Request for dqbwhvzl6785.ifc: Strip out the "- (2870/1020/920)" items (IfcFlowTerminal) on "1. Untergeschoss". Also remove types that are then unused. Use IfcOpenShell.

First a look at what the model holds.

```python
import ifcopenshell
import ifcopenshell.util.element

model = ifcopenshell.open("dqbwhvzl6785.ifc")
print(model.schema)
storey = next(s for s in model.by_type("IfcBuildingStorey") if s.Name == "1. Untergeschoss")
terminals = [e for e in ifcopenshell.util.element.get_decomposition(storey) if e.is_a("IfcFlowTerminal")]
seen = {}
for e in terminals:
    element_type = ifcopenshell.util.element.get_type(e)
    name = element_type.Name if element_type not in (None, e) else None
    seen[name] = seen.get(name, 0) + 1
for name, count in sorted(seen.items(), key=str):
    print(count, "x", name)
```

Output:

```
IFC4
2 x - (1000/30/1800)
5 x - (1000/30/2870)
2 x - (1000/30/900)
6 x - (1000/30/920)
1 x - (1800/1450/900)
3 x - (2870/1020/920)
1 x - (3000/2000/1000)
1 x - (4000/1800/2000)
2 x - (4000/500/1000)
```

```python
import ifcopenshell
import ifcopenshell.api.root
import ifcopenshell.util.element

model = ifcopenshell.open("dqbwhvzl6785.ifc")

storey = next(s for s in model.by_type("IfcBuildingStorey") if s.Name == "1. Untergeschoss")
terminals = [e for e in ifcopenshell.util.element.get_decomposition(storey) if e.is_a("IfcFlowTerminal")]
targets = [e for e in terminals if (t := ifcopenshell.util.element.get_type(e)) not in (None, e) and t.Name == "- (2870/1020/920)"]
types = {ifcopenshell.util.element.get_type(e) for e in targets} - {None, *targets}

for e in targets:
    ifcopenshell.api.root.remove_product(model, product=e)
print(len(targets), "removed")

unused = [t for t in types if not ifcopenshell.util.element.get_types(t)]
for t in unused:
    ifcopenshell.api.root.remove_product(model, product=t)
print(len(unused), "unused types removed")

model.write("dqbwhvzl6785-out.ifc")
```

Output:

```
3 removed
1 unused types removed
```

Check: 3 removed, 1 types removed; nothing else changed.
